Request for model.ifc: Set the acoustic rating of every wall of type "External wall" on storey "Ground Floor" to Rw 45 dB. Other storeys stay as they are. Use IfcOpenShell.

First a look at what the model holds.

```python
import ifcopenshell
import ifcopenshell.util.element

model = ifcopenshell.open("model.ifc")
print(model.schema)
storey = next(s for s in model.by_type("IfcBuildingStorey") if s.Name == "Ground Floor")
walls = [e for e in ifcopenshell.util.element.get_decomposition(storey) if e.is_a("IfcWall")]
seen = {}
for e in walls:
    element_type = ifcopenshell.util.element.get_type(e)
    key = (element_type.Name if element_type != e and element_type else None, ifcopenshell.util.element.get_pset(e, "Pset_WallCommon", "AcousticRating"))
    seen[key] = seen.get(key, 0) + 1
for (name, value), count in sorted(seen.items(), key=str):
    print(count, "x", name, "|", value)
```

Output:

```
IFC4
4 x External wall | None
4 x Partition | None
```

```python
import ifcopenshell
import ifcopenshell.api.pset
import ifcopenshell.util.element

model = ifcopenshell.open("model.ifc")

storey = next(s for s in model.by_type("IfcBuildingStorey") if s.Name == "Ground Floor")
walls = [e for e in ifcopenshell.util.element.get_decomposition(storey) if e.is_a("IfcWall")]

count = 0
for e in walls:
    element_type = ifcopenshell.util.element.get_type(e)
    if element_type in (None, e) or element_type.Name != "External wall":
        continue
    # add_pset returns the element's existing set when there is one.
    pset = ifcopenshell.api.pset.add_pset(model, product=e, name="Pset_WallCommon")
    ifcopenshell.api.pset.edit_pset(model, pset=pset, properties={"AcousticRating": "Rw 45 dB"})
    count += 1

print(count, "walls updated")

model.write("model_edited.ifc")
```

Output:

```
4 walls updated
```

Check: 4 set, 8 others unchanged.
